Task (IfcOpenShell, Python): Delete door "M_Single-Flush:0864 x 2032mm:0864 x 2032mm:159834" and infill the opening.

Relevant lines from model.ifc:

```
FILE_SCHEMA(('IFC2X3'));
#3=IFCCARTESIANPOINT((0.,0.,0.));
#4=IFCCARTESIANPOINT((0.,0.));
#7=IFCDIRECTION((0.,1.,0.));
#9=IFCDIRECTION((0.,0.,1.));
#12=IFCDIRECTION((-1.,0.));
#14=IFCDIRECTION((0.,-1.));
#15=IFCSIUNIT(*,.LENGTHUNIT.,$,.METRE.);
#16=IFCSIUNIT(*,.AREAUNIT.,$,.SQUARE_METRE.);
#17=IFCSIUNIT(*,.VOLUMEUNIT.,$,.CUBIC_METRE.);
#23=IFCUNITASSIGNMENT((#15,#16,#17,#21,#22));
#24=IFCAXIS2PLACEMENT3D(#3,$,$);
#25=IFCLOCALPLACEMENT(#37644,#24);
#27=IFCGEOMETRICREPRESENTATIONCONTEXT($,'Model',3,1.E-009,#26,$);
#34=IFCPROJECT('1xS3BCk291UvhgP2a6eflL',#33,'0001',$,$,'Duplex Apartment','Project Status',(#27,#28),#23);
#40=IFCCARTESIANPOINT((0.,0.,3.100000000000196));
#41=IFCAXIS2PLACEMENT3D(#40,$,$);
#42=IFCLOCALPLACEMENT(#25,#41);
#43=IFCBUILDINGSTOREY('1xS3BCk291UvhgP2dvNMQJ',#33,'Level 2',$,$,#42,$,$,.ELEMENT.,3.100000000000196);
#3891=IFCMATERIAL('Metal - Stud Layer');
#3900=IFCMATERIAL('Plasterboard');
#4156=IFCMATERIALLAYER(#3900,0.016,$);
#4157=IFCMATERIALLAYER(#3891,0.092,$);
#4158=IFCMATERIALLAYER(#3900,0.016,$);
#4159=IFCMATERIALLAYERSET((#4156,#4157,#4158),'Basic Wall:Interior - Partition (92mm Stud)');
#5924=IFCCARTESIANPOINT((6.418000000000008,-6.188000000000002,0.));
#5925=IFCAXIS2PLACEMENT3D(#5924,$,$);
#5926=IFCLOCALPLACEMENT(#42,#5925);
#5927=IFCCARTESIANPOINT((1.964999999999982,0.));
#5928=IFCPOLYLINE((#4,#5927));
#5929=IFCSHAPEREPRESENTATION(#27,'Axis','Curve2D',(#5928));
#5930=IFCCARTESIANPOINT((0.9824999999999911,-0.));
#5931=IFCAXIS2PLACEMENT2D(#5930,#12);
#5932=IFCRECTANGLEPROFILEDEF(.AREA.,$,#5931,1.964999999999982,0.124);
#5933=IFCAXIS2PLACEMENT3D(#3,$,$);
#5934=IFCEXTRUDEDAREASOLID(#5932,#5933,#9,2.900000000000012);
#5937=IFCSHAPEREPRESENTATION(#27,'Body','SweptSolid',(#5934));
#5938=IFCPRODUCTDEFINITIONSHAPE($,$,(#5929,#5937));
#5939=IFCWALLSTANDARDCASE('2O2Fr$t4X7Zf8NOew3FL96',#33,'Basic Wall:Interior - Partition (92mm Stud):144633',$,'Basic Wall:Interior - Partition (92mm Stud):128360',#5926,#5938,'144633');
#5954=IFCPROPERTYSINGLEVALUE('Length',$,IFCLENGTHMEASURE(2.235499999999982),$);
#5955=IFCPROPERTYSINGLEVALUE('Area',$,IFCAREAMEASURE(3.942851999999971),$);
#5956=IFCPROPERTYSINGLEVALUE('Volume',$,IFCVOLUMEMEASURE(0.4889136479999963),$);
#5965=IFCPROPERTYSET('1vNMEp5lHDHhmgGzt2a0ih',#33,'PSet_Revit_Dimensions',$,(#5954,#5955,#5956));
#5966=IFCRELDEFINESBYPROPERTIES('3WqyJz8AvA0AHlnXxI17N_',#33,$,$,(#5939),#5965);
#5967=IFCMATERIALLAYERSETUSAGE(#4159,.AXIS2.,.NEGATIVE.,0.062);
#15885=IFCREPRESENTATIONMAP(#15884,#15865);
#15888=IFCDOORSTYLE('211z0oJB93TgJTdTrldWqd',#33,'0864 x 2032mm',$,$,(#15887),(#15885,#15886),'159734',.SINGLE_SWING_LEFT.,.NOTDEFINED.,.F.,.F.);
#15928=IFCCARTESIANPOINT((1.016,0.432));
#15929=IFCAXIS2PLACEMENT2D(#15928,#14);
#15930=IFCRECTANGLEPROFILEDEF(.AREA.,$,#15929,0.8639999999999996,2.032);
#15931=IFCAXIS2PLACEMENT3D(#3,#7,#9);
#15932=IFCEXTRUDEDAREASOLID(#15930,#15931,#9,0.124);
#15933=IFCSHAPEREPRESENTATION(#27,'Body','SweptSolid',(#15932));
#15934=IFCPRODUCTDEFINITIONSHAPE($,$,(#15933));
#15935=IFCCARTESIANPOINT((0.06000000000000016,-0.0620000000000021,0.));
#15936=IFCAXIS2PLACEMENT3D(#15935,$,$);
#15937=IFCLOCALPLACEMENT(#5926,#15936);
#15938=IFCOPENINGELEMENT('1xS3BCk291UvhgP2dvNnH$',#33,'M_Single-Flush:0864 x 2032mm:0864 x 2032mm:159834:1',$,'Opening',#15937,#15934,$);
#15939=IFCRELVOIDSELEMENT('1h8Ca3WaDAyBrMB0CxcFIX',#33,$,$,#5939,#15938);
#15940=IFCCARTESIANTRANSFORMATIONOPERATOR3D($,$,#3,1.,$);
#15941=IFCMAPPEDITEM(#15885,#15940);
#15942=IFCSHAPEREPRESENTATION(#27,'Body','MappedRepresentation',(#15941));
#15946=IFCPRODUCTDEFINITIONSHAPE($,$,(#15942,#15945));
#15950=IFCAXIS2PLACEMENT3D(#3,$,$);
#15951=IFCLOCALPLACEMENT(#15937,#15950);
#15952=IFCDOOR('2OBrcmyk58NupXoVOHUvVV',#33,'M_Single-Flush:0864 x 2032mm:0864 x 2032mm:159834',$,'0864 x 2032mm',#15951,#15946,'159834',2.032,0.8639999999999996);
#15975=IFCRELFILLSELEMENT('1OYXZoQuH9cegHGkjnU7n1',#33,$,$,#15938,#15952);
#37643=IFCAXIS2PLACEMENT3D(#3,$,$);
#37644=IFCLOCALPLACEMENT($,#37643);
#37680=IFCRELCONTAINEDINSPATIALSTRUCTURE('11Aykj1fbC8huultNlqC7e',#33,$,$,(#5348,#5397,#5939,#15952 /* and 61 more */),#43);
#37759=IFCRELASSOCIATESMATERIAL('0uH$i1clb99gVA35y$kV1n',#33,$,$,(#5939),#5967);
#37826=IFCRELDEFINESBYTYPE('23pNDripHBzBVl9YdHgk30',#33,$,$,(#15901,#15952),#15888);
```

```python
import ifcopenshell
import ifcopenshell.api.feature
import ifcopenshell.api.pset
import ifcopenshell.api.root
import ifcopenshell.geom
import ifcopenshell.util.element
import ifcopenshell.util.shape
import ifcopenshell.util.unit

model = ifcopenshell.open("model.ifc")
area_scale = ifcopenshell.util.unit.calculate_unit_scale(model, "AREAUNIT")
volume_scale = ifcopenshell.util.unit.calculate_unit_scale(model, "VOLUMEUNIT")
settings = ifcopenshell.geom.settings()


def volume(element):
    """Net volume in cubic metres, openings subtracted."""
    shape = ifcopenshell.geom.create_shape(settings, element)
    return ifcopenshell.util.shape.get_volume(shape.geometry)


door = model.by_guid("2OBrcmyk58NupXoVOHUvVV")
opening = door.FillsVoids[0].RelatingOpeningElement
wall = opening.VoidsElements[0].RelatingBuildingElement
before = volume(wall)

ifcopenshell.api.root.remove_product(model, product=door)
ifcopenshell.api.feature.remove_feature(model, feature=opening)

after = volume(wall)
thickness = 0.124  # wall thickness in metres

# Update the wall's stored quantities.
pset = model.by_id(ifcopenshell.util.element.get_pset(wall, "PSet_Revit_Dimensions", should_inherit=False)["id"])
ifcopenshell.api.pset.edit_pset(model, pset=pset, properties={
    "Area": model.create_entity("IfcAreaMeasure", after / thickness / area_scale),
    "Volume": model.create_entity("IfcVolumeMeasure", after / volume_scale),
})

print(f"wall volume {before:.3f} -> {after:.3f} m3")

model.write("model-out.ifc")
```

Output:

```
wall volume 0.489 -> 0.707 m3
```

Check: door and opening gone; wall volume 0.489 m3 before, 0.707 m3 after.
